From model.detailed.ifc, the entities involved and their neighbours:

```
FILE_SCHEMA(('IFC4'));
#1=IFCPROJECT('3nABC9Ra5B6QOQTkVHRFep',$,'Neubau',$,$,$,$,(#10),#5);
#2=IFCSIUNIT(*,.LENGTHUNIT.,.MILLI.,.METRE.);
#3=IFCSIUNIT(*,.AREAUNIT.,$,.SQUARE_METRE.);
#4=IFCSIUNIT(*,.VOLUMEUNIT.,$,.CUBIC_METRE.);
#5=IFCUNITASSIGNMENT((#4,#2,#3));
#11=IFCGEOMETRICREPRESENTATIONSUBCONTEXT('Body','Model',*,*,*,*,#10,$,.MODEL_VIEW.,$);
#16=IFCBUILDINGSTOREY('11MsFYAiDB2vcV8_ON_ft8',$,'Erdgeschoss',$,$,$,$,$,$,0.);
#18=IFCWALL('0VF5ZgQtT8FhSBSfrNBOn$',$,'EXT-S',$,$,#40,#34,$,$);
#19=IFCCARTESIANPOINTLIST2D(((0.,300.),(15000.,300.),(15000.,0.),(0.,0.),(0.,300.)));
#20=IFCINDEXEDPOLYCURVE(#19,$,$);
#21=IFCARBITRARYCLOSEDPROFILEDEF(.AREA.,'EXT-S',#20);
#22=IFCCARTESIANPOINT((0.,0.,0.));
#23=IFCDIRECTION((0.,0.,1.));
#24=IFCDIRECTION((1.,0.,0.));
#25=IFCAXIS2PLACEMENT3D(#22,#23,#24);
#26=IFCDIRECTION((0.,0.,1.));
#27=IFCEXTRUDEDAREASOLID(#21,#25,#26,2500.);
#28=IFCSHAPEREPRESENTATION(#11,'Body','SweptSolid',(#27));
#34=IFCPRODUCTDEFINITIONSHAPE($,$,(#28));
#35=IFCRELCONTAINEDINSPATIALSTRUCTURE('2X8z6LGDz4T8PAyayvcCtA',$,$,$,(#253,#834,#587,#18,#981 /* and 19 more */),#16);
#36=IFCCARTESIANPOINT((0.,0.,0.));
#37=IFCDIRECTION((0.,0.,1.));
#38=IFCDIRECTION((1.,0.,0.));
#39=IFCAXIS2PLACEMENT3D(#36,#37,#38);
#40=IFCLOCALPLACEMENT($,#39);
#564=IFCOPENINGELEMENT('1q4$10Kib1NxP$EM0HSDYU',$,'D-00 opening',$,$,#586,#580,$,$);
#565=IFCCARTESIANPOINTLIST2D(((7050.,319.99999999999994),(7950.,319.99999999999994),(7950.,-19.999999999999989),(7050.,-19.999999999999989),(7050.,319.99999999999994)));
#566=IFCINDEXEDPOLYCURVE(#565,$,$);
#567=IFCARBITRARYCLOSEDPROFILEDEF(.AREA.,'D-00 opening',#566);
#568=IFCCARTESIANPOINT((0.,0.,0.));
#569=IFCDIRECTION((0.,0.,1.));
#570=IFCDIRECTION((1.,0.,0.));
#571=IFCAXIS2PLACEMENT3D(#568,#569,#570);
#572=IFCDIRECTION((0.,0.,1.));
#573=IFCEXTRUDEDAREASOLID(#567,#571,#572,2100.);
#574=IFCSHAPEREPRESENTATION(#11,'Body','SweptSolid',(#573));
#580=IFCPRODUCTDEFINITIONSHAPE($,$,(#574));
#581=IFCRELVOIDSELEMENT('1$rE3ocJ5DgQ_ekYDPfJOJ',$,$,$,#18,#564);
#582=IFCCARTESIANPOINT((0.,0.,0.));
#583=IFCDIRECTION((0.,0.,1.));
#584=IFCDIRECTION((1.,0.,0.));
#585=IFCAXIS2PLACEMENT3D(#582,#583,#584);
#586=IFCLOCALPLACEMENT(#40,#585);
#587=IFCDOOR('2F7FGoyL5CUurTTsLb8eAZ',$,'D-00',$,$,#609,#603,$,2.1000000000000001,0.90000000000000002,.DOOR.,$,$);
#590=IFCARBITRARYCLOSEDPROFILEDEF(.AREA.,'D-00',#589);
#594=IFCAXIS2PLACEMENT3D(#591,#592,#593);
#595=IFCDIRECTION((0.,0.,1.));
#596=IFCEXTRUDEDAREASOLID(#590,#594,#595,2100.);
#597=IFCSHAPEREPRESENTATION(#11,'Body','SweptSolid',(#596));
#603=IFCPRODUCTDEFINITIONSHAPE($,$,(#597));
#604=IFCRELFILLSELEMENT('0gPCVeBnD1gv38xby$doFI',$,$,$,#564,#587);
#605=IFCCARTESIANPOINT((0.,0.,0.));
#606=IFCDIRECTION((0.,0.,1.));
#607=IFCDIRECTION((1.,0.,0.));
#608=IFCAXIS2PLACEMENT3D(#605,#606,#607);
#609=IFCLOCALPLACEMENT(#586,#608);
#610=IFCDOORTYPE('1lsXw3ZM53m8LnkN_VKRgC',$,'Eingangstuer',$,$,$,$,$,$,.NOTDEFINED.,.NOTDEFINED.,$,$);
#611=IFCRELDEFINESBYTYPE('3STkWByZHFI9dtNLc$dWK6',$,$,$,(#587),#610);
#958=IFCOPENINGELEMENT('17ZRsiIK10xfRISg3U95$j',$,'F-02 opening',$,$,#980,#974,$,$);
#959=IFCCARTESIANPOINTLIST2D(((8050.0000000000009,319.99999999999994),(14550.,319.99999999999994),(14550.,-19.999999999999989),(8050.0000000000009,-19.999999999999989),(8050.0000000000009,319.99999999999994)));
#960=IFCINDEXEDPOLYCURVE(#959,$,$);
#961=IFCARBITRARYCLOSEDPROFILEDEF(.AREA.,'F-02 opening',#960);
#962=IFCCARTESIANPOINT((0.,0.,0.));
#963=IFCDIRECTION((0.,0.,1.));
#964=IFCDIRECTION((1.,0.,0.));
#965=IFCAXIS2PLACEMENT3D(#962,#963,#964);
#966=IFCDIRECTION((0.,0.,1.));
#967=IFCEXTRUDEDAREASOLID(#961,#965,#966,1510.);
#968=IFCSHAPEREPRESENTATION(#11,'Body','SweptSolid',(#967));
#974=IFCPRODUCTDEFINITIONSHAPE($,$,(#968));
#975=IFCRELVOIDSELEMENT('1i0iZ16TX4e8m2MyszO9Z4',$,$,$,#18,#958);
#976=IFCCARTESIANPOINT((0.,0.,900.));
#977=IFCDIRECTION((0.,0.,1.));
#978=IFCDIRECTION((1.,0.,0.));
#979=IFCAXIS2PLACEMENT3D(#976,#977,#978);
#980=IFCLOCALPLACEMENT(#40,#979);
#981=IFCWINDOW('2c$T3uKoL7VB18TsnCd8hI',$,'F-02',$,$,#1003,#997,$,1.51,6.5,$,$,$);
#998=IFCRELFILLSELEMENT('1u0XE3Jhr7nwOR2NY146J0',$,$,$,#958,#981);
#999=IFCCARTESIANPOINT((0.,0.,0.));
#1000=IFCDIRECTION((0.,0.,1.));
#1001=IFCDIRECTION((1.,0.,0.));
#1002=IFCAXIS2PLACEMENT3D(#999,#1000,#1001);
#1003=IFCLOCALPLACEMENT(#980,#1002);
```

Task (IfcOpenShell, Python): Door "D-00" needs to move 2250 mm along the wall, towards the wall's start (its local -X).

```python
import ifcopenshell
import ifcopenshell.api.geometry
import ifcopenshell.util.placement
import ifcopenshell.util.unit

model = ifcopenshell.open("model.detailed.ifc")
unit_scale = ifcopenshell.util.unit.calculate_unit_scale(model)

door = model.by_guid("2F7FGoyL5CUurTTsLb8eAZ")
opening = door.FillsVoids[0].RelatingOpeningElement
wall = opening.VoidsElements[0].RelatingBuildingElement

wall_matrix = ifcopenshell.util.placement.get_local_placement(wall.ObjectPlacement)
shift = wall_matrix[:3, 0] * -2.25 / unit_scale
before = ifcopenshell.util.placement.get_local_placement(door.ObjectPlacement)[:3, 3].copy()

# The door is placed relative to its opening, so it follows when the opening moves.
matrix = ifcopenshell.util.placement.get_local_placement(opening.ObjectPlacement)
matrix[:3, 3] += shift
ifcopenshell.api.geometry.edit_object_placement(
    model, product=opening, matrix=matrix, is_si=False, should_transform_children=True
)

after = ifcopenshell.util.placement.get_local_placement(door.ObjectPlacement)[:3, 3]
print("door moved by", (after - before).round(3) + 0.0)

model.write("model.detailed_edited.ifc")
```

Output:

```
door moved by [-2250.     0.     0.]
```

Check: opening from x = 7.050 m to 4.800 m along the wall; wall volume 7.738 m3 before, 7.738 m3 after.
